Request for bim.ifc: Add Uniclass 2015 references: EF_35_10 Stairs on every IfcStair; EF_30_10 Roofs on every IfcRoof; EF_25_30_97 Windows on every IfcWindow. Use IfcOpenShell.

First a look at what the model holds.

```python
import ifcopenshell

model = ifcopenshell.open("bim.ifc")
print(model.schema)
print("classifications:", [c.Name for c in model.by_type("IfcClassification")])
for ifc_class in ("IfcDoor", "IfcRoof", "IfcStair", "IfcWall", "IfcWindow"):
    print(ifc_class, len(model.by_type(ifc_class)))
```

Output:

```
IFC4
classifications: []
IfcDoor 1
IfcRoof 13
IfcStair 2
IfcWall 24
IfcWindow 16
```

```python
import ifcopenshell
import ifcopenshell.api.classification

model = ifcopenshell.open("bim.ifc")

system = ifcopenshell.api.classification.add_classification(model, classification="Uniclass 2015")

codes = {
    "IfcStair": ("EF_35_10", "Stairs"),
    "IfcRoof": ("EF_30_10", "Roofs"),
    "IfcWindow": ("EF_25_30_97", "Windows"),
}
for ifc_class, (code, name) in codes.items():
    products = model.by_type(ifc_class)
    ifcopenshell.api.classification.add_reference(
        model, products=products, classification=system, identification=code, name=name
    )
    print(code, len(products))

model.write("bim_updated.ifc")
```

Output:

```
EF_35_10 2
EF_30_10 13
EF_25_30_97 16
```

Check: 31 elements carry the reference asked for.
